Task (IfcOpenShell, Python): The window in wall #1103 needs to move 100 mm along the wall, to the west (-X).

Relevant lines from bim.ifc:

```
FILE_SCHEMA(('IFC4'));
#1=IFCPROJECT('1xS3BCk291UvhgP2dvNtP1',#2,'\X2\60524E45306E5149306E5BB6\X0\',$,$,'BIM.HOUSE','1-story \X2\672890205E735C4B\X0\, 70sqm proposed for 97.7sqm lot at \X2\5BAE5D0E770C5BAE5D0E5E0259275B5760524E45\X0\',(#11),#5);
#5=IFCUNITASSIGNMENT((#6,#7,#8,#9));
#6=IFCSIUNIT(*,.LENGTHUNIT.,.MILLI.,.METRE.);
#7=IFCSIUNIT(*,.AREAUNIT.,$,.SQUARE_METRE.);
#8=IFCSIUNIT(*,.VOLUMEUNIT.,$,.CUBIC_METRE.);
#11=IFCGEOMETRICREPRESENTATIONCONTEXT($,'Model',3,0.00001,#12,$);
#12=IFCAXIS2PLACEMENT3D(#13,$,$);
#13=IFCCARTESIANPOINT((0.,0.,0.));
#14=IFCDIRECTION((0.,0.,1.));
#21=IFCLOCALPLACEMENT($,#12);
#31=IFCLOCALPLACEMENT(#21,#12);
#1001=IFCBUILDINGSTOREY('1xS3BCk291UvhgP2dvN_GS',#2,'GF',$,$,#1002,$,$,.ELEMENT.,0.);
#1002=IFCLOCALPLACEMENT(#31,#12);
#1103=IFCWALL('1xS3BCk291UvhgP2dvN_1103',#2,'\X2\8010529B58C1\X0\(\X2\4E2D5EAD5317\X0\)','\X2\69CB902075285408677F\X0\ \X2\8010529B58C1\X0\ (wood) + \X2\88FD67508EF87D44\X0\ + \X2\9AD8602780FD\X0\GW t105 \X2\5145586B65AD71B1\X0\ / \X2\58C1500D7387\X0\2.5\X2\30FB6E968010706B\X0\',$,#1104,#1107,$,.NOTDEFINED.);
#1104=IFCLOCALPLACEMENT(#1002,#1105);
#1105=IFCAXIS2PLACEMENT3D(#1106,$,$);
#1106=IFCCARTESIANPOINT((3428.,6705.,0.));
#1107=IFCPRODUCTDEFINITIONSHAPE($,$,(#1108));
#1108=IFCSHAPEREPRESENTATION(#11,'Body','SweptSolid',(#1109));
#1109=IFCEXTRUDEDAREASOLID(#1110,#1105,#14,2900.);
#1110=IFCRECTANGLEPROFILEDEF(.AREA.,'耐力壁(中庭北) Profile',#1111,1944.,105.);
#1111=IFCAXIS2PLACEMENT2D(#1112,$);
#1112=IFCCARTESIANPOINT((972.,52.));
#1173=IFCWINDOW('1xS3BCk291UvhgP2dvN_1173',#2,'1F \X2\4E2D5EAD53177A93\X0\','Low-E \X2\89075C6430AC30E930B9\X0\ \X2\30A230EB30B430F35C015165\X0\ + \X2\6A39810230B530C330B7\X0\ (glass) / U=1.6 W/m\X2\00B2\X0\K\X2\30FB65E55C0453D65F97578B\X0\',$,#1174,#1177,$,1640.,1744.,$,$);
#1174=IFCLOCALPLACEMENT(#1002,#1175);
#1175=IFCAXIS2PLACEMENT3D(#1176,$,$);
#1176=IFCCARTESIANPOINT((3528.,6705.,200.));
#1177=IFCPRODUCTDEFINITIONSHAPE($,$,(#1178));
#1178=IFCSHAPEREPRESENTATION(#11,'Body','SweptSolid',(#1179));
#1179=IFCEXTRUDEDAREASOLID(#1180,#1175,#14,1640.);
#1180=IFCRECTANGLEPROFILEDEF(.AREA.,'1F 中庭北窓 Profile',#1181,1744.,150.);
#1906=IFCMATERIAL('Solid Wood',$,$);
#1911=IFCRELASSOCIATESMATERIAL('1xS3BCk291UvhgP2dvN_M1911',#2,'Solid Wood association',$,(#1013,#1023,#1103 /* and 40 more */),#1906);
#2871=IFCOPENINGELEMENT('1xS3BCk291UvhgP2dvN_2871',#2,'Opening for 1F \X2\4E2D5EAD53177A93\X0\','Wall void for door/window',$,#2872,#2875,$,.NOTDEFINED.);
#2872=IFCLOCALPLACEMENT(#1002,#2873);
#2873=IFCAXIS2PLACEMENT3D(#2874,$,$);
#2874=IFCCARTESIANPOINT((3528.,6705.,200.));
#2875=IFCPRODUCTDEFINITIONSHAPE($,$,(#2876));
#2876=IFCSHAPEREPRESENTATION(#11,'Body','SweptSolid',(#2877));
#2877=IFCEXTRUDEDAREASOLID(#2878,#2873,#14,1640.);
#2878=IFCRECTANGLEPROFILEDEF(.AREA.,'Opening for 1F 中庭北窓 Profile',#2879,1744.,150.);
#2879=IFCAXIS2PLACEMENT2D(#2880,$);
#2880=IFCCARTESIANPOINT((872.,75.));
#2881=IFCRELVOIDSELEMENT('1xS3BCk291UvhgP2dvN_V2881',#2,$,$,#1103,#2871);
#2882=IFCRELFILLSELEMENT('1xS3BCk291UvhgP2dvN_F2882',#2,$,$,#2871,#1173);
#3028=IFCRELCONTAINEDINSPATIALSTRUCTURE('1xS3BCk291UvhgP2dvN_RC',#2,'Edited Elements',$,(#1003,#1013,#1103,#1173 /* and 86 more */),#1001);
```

```python
import ifcopenshell
import ifcopenshell.api.geometry
import ifcopenshell.util.placement
import ifcopenshell.util.unit

model = ifcopenshell.open("bim.ifc")
unit_scale = ifcopenshell.util.unit.calculate_unit_scale(model)

window = model.by_guid("1xS3BCk291UvhgP2dvN_1173")
opening = window.FillsVoids[0].RelatingOpeningElement
wall = opening.VoidsElements[0].RelatingBuildingElement

wall_matrix = ifcopenshell.util.placement.get_local_placement(wall.ObjectPlacement)
shift = wall_matrix[:3, 0] * -0.1 / unit_scale
before = ifcopenshell.util.placement.get_local_placement(window.ObjectPlacement)[:3, 3].copy()

# The window is not placed relative to its opening, so move both.
for product in (opening, window):
    matrix = ifcopenshell.util.placement.get_local_placement(product.ObjectPlacement)
    matrix[:3, 3] += shift
    ifcopenshell.api.geometry.edit_object_placement(model, product=product, matrix=matrix, is_si=False)

after = ifcopenshell.util.placement.get_local_placement(window.ObjectPlacement)[:3, 3]
print("window moved by", (after - before).round(3) + 0.0)

model.write("bim_edited.ifc")
```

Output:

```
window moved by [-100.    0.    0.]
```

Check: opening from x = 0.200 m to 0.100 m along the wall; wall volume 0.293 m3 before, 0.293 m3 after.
